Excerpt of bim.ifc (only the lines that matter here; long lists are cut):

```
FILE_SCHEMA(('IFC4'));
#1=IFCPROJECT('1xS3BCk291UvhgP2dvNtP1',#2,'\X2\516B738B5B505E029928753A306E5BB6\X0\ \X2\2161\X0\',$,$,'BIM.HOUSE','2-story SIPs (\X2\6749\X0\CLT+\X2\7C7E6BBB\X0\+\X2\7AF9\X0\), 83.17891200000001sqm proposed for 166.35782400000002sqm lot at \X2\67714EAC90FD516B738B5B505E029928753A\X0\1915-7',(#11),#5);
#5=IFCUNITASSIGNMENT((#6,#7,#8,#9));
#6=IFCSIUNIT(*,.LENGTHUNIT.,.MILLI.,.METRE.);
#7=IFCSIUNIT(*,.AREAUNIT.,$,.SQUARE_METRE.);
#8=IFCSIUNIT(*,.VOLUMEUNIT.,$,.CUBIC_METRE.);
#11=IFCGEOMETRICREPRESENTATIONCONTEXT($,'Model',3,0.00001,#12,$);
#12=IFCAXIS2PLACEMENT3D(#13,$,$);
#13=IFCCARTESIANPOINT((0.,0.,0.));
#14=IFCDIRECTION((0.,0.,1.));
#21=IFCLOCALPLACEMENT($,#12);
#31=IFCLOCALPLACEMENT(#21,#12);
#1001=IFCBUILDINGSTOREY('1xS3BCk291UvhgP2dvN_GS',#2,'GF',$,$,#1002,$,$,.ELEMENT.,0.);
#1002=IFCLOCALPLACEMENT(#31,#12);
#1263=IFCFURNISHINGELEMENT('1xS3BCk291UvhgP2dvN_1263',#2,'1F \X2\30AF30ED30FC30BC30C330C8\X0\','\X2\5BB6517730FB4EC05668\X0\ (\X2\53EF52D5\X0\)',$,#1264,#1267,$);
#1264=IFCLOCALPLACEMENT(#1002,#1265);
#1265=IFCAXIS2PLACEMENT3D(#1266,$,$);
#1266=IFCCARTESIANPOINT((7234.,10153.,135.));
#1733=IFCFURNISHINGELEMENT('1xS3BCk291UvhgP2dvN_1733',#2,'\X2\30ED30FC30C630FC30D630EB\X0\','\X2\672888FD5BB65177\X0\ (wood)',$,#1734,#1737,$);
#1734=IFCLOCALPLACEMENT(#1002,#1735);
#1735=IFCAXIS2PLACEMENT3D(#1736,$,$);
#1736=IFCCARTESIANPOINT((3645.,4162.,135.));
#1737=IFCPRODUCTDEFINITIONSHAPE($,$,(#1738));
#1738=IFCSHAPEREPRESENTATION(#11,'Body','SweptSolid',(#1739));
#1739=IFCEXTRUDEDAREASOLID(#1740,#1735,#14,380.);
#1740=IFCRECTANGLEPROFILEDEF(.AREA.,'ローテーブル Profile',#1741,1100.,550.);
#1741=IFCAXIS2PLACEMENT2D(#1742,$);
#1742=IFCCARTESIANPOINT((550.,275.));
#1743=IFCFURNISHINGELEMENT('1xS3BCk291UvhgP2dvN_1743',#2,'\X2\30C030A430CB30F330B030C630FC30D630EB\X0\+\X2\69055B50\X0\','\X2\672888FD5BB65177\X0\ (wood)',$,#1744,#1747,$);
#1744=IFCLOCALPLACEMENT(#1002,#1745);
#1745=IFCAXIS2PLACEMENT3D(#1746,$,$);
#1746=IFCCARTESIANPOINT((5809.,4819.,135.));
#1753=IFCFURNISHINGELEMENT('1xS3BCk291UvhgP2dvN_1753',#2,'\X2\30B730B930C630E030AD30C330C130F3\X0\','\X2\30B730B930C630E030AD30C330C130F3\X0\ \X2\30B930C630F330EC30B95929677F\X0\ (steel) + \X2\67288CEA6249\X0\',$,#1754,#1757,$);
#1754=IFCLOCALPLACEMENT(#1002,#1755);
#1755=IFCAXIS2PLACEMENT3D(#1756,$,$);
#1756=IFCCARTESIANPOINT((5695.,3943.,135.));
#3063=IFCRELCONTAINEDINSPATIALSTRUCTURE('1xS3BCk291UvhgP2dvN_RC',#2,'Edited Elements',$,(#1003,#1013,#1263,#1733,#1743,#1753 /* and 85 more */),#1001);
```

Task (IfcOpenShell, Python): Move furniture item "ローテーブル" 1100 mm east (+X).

```python
import ifcopenshell
import ifcopenshell.api.geometry
import ifcopenshell.util.placement

model = ifcopenshell.open("bim.ifc")

item = model.by_id(1733)
matrix = ifcopenshell.util.placement.get_local_placement(item.ObjectPlacement)
matrix[0, 3] += 1100.0
ifcopenshell.api.geometry.edit_object_placement(model, product=item, matrix=matrix, is_si=False)

print(ifcopenshell.util.placement.get_local_placement(item.ObjectPlacement).round(3) + 0.0)

model.write("bim_v2.ifc")
```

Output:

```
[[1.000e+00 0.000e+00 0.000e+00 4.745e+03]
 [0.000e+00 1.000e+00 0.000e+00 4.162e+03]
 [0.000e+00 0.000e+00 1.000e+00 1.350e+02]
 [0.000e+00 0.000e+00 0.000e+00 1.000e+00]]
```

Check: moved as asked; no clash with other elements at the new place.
